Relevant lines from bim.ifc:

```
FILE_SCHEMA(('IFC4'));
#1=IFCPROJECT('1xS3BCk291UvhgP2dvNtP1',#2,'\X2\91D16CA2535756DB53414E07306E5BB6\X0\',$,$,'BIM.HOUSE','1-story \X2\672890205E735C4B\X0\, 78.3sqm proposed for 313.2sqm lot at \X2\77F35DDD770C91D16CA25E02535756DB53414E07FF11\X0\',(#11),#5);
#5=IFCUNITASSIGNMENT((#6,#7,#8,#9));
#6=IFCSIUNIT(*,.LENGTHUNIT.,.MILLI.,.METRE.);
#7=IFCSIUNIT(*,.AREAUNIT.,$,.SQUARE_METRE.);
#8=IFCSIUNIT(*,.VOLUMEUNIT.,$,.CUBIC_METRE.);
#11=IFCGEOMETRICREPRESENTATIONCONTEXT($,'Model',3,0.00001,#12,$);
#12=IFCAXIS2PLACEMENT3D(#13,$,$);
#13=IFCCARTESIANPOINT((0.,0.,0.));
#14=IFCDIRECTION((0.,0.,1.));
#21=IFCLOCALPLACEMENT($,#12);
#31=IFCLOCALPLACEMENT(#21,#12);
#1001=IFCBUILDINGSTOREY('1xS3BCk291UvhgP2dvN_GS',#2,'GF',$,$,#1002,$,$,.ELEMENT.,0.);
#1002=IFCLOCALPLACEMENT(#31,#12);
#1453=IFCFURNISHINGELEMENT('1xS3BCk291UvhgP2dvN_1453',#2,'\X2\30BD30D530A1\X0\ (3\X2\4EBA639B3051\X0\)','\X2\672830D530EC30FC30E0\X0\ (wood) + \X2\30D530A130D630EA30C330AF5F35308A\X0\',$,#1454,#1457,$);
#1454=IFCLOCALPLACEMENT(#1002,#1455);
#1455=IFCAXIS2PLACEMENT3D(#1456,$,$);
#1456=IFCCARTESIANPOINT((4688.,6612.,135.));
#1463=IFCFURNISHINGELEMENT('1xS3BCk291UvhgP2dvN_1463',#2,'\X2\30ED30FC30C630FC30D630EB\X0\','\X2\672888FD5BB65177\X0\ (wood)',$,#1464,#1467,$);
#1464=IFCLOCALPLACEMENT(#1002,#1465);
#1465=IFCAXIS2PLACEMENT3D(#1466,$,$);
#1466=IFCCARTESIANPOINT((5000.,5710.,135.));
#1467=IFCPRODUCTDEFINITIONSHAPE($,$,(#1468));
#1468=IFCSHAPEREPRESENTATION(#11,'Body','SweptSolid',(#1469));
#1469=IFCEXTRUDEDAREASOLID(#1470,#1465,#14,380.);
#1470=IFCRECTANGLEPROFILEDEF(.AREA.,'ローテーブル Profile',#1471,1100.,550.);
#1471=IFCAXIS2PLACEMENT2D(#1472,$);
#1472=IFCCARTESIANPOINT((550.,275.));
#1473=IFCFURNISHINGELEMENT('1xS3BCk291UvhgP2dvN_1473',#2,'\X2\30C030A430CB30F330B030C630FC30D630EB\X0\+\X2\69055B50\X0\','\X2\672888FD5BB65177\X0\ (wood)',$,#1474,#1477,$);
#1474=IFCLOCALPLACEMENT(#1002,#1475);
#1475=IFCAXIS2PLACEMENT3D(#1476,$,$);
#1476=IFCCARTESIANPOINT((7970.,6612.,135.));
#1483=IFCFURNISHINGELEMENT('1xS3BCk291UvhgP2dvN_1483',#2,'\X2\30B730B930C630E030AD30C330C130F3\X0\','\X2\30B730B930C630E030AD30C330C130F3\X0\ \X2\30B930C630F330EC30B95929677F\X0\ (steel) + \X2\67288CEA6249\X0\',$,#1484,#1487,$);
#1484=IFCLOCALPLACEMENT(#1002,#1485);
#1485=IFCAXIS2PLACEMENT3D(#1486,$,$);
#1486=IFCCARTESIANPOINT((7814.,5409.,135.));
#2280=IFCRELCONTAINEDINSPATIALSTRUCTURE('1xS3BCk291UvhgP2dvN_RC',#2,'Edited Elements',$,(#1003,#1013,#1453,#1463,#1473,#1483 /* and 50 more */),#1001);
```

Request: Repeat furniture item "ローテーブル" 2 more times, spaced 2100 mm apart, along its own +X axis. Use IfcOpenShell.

```python
import ifcopenshell
import ifcopenshell.api.geometry
import ifcopenshell.api.root
import ifcopenshell.util.element
import ifcopenshell.util.placement
import ifcopenshell.util.unit

model = ifcopenshell.open("bim.ifc")
unit_scale = ifcopenshell.util.unit.calculate_unit_scale(model)


def reuse_history(source, copy):
    """copy_class also copies each property set's owner history, people and application; keep the originals."""
    for rel in copy.IsDefinedBy:
        if rel.is_a("IfcRelDefinesByProperties") and (history := rel.RelatingPropertyDefinition.OwnerHistory):
            rel.RelatingPropertyDefinition.OwnerHistory = source.OwnerHistory
            ifcopenshell.util.element.remove_deep2(model, history)


source = model.by_guid("1xS3BCk291UvhgP2dvN_1463")
base = ifcopenshell.util.placement.get_local_placement(source.ObjectPlacement)
step = base[:3, 0] * 2.1 / unit_scale

for i in range(1, 3):
    copy = ifcopenshell.api.root.copy_class(model, product=source)
    copy.Representation = ifcopenshell.util.element.copy_deep(
        model, source.Representation, exclude=["IfcGeometricRepresentationContext", "IfcRepresentationMap"]
    )
    reuse_history(source, copy)
    matrix = base.copy()
    matrix[:3, 3] += i * step
    print("added at", matrix[:3, 3].round(3) + 0.0)
    ifcopenshell.api.geometry.edit_object_placement(model, product=copy, matrix=matrix, is_si=False)

model.write("bim_rev.ifc")
```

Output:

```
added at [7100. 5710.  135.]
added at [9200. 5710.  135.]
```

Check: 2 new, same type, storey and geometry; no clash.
